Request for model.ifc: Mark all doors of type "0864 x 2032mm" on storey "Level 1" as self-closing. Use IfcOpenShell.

First a look at what the model holds.

```python
import ifcopenshell
import ifcopenshell.util.element

model = ifcopenshell.open("model.ifc")
print(model.schema)
storey = next(s for s in model.by_type("IfcBuildingStorey") if s.Name == "Level 1")
doors = [e for e in ifcopenshell.util.element.get_decomposition(storey) if e.is_a("IfcDoor")]
seen = {}
for e in doors:
    element_type = ifcopenshell.util.element.get_type(e)
    key = (element_type.Name if element_type != e and element_type else None, ifcopenshell.util.element.get_pset(e, "Pset_DoorCommon", "SelfClosing"))
    seen[key] = seen.get(key, 0) + 1
for (name, value), count in sorted(seen.items(), key=str):
    print(count, "x", name, "|", value)
```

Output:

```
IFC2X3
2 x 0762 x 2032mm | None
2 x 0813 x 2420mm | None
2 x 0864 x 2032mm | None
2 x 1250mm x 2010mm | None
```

```python
import ifcopenshell
import ifcopenshell.api.pset
import ifcopenshell.util.element

model = ifcopenshell.open("model.ifc")

storey = next(s for s in model.by_type("IfcBuildingStorey") if s.Name == "Level 1")
doors = [e for e in ifcopenshell.util.element.get_decomposition(storey) if e.is_a("IfcDoor")]

count = 0
for e in doors:
    element_type = ifcopenshell.util.element.get_type(e)
    if element_type in (None, e) or element_type.Name != "0864 x 2032mm":
        continue
    # add_pset returns the element's existing set when there is one.
    pset = ifcopenshell.api.pset.add_pset(model, product=e, name="Pset_DoorCommon")
    ifcopenshell.api.pset.edit_pset(model, pset=pset, properties={"SelfClosing": True})
    count += 1

print(count, "doors updated")

model.write("model_updated.ifc")
```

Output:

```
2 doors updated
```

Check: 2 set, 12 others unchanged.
